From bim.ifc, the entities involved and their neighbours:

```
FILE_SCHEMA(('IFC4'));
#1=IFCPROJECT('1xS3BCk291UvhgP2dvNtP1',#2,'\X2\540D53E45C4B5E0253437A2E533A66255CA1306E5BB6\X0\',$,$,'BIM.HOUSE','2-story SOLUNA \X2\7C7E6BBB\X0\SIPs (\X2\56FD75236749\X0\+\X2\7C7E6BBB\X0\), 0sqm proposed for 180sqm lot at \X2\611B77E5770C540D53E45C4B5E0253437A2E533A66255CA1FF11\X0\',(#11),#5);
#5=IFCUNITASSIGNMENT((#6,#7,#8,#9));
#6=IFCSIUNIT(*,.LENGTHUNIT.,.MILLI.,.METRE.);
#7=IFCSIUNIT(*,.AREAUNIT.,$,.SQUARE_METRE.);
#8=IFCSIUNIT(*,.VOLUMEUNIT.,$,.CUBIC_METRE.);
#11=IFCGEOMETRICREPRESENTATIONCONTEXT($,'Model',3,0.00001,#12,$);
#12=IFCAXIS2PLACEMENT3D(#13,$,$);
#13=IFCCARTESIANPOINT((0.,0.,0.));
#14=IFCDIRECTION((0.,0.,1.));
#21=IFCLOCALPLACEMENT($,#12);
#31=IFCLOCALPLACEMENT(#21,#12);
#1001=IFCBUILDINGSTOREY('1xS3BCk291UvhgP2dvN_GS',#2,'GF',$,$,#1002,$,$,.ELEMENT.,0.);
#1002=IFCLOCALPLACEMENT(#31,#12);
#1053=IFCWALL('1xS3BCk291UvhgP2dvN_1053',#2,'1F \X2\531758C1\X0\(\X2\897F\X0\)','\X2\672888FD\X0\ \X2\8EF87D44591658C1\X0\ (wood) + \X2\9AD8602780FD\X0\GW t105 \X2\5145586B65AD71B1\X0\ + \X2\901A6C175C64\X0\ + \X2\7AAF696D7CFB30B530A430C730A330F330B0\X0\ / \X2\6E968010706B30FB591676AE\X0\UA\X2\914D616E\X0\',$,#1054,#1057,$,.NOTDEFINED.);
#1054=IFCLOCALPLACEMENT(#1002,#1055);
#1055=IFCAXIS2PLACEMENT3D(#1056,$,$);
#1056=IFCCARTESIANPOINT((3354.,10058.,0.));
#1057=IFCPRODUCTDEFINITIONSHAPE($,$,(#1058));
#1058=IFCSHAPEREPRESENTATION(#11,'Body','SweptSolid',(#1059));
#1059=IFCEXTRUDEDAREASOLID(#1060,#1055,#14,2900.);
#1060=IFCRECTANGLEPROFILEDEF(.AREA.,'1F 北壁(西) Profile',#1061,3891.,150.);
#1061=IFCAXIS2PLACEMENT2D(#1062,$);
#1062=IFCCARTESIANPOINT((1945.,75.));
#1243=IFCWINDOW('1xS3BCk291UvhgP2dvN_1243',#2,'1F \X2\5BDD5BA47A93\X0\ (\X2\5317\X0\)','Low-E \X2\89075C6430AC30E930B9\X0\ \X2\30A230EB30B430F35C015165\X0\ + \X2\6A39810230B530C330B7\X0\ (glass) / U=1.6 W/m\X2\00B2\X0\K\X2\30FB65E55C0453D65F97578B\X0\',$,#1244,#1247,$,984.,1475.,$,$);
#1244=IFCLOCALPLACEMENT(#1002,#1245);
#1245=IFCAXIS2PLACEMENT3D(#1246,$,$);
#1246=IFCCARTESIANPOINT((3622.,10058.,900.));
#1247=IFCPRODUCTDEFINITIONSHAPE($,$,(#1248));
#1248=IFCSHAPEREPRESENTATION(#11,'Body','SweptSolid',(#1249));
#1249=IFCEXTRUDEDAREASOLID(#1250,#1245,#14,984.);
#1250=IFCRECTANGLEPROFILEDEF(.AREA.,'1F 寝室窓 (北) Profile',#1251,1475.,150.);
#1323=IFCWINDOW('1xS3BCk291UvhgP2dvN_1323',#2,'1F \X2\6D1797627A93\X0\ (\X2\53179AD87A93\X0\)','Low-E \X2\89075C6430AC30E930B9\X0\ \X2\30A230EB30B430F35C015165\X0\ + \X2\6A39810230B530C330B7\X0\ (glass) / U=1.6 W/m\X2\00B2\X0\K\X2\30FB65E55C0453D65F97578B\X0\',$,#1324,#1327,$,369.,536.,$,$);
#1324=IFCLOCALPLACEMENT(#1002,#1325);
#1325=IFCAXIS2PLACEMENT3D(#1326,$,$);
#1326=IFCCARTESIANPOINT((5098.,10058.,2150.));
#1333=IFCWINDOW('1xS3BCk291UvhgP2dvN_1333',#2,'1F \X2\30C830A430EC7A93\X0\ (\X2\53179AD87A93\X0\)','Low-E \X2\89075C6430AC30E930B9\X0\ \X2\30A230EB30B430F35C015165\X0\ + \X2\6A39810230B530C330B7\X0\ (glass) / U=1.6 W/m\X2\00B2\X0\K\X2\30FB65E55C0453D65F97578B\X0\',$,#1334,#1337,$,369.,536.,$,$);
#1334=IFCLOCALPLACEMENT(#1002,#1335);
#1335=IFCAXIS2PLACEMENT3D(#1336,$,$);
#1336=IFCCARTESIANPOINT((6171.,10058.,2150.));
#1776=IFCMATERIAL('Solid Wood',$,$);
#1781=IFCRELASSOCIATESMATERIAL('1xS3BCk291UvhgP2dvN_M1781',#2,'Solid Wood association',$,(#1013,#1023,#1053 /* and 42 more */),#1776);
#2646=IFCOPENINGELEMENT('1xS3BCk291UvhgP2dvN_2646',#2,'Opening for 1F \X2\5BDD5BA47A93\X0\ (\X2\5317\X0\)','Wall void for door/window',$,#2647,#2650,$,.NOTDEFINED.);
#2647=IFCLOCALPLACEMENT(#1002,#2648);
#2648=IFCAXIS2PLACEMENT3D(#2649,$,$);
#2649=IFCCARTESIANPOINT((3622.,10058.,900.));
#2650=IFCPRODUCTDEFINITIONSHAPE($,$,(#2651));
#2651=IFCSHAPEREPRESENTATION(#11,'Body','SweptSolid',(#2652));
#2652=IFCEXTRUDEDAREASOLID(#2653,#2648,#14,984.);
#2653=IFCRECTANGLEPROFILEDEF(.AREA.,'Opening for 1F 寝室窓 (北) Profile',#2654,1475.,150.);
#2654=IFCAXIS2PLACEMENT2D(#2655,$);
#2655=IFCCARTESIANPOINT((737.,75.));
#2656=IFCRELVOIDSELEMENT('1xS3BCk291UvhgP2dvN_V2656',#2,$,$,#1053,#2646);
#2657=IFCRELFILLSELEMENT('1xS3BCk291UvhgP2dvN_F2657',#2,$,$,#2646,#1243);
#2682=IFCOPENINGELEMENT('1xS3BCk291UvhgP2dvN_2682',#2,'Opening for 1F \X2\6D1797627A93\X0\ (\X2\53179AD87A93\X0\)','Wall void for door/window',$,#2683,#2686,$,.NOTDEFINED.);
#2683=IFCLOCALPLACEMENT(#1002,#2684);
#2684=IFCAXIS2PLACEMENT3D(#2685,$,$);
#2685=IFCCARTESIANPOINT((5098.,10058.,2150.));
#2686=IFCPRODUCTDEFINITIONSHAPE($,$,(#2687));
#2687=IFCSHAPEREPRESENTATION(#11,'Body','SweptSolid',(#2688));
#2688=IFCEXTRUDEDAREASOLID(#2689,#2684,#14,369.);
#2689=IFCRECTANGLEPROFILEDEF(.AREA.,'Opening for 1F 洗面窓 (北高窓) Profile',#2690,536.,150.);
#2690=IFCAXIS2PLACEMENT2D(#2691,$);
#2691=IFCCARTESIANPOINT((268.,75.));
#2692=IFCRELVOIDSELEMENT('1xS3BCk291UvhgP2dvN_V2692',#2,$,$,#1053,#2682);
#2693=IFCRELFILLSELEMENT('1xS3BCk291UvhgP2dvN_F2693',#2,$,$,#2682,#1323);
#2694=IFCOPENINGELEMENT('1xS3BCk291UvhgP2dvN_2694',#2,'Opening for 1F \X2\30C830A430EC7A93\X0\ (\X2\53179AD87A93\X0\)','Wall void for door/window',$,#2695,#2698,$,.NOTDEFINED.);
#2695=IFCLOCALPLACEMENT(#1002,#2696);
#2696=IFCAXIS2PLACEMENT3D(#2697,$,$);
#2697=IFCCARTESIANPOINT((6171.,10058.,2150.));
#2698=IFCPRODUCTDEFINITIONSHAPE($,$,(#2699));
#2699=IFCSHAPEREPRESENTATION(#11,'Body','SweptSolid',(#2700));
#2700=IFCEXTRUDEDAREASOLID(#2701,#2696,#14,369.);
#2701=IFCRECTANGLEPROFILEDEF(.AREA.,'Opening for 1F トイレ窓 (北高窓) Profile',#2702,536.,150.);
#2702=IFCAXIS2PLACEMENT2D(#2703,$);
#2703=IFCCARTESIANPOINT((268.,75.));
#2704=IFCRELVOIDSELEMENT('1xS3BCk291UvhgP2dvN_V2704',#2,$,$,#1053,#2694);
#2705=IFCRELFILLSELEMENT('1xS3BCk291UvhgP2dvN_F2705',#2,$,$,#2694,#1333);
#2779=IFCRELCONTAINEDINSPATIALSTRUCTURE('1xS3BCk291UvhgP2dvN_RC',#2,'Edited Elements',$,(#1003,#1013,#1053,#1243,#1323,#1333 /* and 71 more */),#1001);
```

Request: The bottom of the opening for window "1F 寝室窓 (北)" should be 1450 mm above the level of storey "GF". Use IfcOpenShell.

```python
import numpy as np
import ifcopenshell
import ifcopenshell.api.geometry
import ifcopenshell.geom
import ifcopenshell.util.element
import ifcopenshell.util.placement
import ifcopenshell.util.shape
import ifcopenshell.util.unit

model = ifcopenshell.open("bim.ifc")
unit_scale = ifcopenshell.util.unit.calculate_unit_scale(model)

window = model.by_guid("1xS3BCk291UvhgP2dvN_1243")
opening = window.FillsVoids[0].RelatingOpeningElement
storey = ifcopenshell.util.element.get_container(window, ifc_class="IfcBuildingStorey")
level = ifcopenshell.util.placement.get_local_placement(storey.ObjectPlacement)[2, 3]

# The opening's origin need not be at the sill, so measure its lowest point.
shape = ifcopenshell.geom.create_shape(ifcopenshell.geom.settings(), opening)
bottom = ifcopenshell.util.shape.get_shape_bottom_elevation(shape, shape.geometry) / unit_scale
dz = level + 1450.0 - bottom

shift = np.array([0.0, 0.0, dz])
# The window is not placed relative to its opening, so move both.
for product in (opening, window):
    matrix = ifcopenshell.util.placement.get_local_placement(product.ObjectPlacement)
    matrix[:3, 3] += shift
    ifcopenshell.api.geometry.edit_object_placement(model, product=product, matrix=matrix, is_si=False)

print(f"moved by {dz * unit_scale:+.3f} m")

model.write("bim-out.ifc")
```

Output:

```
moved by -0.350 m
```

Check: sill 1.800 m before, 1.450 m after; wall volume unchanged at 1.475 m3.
